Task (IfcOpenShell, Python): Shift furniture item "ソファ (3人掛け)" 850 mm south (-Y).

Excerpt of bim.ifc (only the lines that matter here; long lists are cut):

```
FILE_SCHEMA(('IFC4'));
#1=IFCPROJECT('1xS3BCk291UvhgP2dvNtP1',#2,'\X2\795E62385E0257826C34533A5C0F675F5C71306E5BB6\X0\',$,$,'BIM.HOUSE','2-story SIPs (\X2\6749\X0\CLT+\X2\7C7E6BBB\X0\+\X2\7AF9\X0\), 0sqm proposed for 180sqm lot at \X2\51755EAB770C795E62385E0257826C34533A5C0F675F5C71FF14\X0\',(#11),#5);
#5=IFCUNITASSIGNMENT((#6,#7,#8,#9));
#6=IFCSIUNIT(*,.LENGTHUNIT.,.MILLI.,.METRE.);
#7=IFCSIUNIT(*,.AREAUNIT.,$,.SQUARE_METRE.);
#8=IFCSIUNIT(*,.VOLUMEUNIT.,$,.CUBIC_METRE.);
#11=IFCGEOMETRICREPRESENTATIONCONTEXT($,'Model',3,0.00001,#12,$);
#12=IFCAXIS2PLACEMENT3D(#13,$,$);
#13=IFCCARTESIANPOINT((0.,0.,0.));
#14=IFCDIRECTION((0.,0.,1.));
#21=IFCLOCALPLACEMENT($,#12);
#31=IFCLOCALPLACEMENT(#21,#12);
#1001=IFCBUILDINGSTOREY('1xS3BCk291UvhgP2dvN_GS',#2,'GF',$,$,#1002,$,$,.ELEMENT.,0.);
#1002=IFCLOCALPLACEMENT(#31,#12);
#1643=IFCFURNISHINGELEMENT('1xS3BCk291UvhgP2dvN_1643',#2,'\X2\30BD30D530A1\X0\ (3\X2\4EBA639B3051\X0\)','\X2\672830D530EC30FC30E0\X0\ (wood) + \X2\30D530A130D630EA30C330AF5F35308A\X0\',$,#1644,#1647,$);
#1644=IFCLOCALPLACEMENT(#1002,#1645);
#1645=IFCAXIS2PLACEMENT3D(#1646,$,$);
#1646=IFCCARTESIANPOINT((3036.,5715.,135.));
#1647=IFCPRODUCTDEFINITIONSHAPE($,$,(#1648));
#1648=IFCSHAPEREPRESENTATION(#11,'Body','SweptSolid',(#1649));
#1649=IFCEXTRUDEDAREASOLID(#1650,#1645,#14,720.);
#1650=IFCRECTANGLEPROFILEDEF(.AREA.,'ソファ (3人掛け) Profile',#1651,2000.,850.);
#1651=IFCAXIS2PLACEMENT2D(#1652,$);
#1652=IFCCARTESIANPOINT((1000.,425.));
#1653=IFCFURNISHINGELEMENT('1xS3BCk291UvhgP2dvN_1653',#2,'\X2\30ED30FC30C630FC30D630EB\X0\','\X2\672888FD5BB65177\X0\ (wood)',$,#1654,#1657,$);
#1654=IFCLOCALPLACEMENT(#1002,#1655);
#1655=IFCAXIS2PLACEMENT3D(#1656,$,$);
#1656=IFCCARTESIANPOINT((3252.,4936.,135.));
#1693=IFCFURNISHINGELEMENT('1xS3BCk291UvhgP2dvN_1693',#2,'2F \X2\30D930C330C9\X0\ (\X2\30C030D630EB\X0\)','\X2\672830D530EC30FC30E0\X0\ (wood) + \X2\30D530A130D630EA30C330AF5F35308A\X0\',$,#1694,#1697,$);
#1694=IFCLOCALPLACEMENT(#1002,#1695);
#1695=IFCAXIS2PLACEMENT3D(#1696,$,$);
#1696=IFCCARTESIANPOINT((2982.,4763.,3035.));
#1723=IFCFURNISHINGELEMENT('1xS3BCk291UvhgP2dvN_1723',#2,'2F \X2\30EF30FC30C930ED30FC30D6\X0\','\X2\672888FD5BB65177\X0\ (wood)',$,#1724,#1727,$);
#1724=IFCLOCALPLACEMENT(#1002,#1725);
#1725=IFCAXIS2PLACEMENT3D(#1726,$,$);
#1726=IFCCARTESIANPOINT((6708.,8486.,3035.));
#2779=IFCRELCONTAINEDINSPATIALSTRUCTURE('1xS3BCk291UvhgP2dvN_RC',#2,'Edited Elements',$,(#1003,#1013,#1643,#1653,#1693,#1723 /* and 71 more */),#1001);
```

```python
import ifcopenshell
import ifcopenshell.api.geometry
import ifcopenshell.util.placement
import ifcopenshell.util.unit

model = ifcopenshell.open("bim.ifc")
unit_scale = ifcopenshell.util.unit.calculate_unit_scale(model)

item = model.by_guid("1xS3BCk291UvhgP2dvN_1643")
matrix = ifcopenshell.util.placement.get_local_placement(item.ObjectPlacement)
matrix[1, 3] -= 0.85 / unit_scale
ifcopenshell.api.geometry.edit_object_placement(model, product=item, matrix=matrix, is_si=False)

print(ifcopenshell.util.placement.get_local_placement(item.ObjectPlacement).round(3) + 0.0)

model.write("bim-out.ifc")
```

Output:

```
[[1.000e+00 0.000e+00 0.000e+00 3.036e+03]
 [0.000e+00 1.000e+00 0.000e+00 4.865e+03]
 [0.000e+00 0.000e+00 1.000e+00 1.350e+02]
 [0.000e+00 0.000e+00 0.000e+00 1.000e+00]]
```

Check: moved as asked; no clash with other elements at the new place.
